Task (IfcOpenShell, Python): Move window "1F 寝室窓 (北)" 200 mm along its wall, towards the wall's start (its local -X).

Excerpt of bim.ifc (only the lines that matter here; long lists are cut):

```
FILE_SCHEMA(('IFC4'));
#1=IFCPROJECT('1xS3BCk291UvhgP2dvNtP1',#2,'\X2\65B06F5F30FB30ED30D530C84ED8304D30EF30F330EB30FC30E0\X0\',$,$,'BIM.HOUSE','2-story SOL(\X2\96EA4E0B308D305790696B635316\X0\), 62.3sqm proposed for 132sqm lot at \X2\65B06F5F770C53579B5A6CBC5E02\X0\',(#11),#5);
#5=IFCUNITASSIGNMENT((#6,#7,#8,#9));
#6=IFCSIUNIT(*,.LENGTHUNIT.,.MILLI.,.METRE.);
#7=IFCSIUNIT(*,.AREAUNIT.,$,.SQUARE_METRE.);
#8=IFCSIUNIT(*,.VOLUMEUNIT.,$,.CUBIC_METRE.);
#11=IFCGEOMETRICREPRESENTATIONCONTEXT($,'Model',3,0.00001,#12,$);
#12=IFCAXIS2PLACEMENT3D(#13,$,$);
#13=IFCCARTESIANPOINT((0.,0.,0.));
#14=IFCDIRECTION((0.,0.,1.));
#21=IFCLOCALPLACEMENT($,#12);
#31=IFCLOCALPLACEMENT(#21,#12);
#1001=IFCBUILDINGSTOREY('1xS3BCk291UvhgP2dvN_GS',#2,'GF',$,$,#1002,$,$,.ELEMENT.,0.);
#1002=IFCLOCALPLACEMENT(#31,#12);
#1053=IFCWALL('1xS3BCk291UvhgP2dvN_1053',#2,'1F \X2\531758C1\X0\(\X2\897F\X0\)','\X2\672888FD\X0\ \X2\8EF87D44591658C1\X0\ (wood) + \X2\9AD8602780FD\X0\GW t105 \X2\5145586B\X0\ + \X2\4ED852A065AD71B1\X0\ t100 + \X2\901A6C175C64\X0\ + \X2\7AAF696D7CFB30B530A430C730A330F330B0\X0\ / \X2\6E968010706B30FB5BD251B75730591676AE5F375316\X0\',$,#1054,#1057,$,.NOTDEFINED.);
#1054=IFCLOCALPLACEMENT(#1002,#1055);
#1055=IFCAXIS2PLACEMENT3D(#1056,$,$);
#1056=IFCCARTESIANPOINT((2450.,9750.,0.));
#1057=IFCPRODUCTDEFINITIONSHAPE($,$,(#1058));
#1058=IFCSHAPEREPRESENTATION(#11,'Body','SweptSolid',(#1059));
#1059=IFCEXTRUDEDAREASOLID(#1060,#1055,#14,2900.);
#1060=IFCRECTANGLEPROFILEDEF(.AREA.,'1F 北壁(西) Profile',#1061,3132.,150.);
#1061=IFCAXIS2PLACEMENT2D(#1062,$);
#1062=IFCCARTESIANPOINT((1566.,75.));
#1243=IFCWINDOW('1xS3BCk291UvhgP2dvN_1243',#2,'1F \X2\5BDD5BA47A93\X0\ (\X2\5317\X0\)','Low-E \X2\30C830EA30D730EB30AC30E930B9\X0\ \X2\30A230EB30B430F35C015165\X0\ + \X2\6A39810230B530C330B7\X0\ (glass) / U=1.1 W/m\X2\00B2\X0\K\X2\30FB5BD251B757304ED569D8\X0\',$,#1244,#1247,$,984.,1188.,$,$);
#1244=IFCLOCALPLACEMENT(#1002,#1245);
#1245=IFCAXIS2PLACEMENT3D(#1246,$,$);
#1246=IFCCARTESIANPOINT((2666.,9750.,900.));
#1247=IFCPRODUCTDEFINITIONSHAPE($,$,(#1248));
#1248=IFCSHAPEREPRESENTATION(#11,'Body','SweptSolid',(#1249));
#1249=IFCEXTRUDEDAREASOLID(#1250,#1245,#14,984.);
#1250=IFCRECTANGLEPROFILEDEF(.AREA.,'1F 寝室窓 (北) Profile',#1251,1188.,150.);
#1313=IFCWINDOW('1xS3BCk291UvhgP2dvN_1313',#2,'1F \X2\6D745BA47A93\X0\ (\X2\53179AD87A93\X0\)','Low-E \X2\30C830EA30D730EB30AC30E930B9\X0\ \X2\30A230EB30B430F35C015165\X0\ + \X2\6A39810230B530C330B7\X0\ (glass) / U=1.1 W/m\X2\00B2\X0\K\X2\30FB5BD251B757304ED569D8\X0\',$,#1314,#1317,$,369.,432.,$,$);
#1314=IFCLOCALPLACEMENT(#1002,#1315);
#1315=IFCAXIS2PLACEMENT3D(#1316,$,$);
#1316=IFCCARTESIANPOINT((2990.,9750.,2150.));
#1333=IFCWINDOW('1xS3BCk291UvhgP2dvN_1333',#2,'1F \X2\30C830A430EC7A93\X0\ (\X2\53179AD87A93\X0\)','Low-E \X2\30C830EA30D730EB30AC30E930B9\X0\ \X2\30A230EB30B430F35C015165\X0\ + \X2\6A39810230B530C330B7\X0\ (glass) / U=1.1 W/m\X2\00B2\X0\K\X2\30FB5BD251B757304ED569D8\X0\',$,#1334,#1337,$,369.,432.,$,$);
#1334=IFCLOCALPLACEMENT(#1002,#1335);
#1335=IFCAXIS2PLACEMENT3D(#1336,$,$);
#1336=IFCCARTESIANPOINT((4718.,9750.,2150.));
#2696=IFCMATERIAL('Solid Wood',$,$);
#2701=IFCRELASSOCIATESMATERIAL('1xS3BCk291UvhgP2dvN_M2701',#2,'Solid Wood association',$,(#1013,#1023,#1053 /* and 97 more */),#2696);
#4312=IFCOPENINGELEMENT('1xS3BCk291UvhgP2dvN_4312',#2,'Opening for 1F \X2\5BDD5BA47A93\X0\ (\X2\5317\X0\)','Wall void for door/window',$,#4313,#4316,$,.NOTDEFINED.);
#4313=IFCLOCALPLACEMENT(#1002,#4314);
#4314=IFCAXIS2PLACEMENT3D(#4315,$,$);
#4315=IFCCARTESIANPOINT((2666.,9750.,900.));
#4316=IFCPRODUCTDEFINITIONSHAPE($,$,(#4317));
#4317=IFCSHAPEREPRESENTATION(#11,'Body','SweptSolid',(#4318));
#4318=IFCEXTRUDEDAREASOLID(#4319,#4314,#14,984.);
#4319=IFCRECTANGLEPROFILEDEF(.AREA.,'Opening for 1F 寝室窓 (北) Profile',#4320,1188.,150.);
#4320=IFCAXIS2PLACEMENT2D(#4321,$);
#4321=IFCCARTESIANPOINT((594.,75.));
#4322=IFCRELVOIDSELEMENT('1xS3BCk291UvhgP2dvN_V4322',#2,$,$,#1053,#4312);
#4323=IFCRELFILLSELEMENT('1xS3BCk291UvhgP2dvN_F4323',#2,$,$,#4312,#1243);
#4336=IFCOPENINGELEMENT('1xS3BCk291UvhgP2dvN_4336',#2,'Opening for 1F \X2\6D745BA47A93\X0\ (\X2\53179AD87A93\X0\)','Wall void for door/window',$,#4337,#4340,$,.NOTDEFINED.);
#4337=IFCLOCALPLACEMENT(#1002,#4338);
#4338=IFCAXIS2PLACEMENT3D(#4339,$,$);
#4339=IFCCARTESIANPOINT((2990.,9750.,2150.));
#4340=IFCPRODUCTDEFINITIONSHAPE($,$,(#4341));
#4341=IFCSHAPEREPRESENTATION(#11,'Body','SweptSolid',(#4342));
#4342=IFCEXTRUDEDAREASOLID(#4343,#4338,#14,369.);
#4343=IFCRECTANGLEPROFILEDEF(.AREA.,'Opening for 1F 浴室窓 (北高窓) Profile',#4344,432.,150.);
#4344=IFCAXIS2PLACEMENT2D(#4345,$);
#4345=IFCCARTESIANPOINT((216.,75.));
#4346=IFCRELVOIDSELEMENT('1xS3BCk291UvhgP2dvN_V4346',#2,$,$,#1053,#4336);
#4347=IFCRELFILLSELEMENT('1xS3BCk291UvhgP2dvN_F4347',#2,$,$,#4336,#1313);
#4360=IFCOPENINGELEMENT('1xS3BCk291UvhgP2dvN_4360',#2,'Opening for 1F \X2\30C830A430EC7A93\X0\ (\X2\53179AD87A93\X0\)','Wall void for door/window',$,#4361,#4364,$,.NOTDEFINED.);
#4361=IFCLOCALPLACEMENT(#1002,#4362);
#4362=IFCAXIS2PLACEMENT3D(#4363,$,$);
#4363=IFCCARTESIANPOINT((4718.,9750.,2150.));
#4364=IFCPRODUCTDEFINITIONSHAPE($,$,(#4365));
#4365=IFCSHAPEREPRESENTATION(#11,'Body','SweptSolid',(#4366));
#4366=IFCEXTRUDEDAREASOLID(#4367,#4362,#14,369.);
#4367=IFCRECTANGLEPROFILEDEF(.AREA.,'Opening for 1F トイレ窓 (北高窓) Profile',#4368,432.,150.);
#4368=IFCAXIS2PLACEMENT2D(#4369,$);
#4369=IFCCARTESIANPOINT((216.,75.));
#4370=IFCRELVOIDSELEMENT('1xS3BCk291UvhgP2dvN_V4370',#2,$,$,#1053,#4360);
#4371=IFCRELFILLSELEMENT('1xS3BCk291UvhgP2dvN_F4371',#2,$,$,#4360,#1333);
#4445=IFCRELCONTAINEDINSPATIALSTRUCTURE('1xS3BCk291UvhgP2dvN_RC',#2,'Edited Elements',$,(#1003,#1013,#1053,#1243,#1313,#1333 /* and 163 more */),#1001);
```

```python
import ifcopenshell
import ifcopenshell.api.geometry
import ifcopenshell.util.placement
import ifcopenshell.util.unit

model = ifcopenshell.open("bim.ifc")
unit_scale = ifcopenshell.util.unit.calculate_unit_scale(model)

window = model.by_guid("1xS3BCk291UvhgP2dvN_1243")
opening = window.FillsVoids[0].RelatingOpeningElement
wall = opening.VoidsElements[0].RelatingBuildingElement

wall_matrix = ifcopenshell.util.placement.get_local_placement(wall.ObjectPlacement)
shift = wall_matrix[:3, 0] * -0.2 / unit_scale
before = ifcopenshell.util.placement.get_local_placement(window.ObjectPlacement)[:3, 3].copy()

# The window is not placed relative to its opening, so move both.
for product in (opening, window):
    matrix = ifcopenshell.util.placement.get_local_placement(product.ObjectPlacement)
    matrix[:3, 3] += shift
    ifcopenshell.api.geometry.edit_object_placement(model, product=product, matrix=matrix, is_si=False)

after = ifcopenshell.util.placement.get_local_placement(window.ObjectPlacement)[:3, 3]
print("window moved by", (after - before).round(3) + 0.0)

model.write("bim_edited.ifc")
```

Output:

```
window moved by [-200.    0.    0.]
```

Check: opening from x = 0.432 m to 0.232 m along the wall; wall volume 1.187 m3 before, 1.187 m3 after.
